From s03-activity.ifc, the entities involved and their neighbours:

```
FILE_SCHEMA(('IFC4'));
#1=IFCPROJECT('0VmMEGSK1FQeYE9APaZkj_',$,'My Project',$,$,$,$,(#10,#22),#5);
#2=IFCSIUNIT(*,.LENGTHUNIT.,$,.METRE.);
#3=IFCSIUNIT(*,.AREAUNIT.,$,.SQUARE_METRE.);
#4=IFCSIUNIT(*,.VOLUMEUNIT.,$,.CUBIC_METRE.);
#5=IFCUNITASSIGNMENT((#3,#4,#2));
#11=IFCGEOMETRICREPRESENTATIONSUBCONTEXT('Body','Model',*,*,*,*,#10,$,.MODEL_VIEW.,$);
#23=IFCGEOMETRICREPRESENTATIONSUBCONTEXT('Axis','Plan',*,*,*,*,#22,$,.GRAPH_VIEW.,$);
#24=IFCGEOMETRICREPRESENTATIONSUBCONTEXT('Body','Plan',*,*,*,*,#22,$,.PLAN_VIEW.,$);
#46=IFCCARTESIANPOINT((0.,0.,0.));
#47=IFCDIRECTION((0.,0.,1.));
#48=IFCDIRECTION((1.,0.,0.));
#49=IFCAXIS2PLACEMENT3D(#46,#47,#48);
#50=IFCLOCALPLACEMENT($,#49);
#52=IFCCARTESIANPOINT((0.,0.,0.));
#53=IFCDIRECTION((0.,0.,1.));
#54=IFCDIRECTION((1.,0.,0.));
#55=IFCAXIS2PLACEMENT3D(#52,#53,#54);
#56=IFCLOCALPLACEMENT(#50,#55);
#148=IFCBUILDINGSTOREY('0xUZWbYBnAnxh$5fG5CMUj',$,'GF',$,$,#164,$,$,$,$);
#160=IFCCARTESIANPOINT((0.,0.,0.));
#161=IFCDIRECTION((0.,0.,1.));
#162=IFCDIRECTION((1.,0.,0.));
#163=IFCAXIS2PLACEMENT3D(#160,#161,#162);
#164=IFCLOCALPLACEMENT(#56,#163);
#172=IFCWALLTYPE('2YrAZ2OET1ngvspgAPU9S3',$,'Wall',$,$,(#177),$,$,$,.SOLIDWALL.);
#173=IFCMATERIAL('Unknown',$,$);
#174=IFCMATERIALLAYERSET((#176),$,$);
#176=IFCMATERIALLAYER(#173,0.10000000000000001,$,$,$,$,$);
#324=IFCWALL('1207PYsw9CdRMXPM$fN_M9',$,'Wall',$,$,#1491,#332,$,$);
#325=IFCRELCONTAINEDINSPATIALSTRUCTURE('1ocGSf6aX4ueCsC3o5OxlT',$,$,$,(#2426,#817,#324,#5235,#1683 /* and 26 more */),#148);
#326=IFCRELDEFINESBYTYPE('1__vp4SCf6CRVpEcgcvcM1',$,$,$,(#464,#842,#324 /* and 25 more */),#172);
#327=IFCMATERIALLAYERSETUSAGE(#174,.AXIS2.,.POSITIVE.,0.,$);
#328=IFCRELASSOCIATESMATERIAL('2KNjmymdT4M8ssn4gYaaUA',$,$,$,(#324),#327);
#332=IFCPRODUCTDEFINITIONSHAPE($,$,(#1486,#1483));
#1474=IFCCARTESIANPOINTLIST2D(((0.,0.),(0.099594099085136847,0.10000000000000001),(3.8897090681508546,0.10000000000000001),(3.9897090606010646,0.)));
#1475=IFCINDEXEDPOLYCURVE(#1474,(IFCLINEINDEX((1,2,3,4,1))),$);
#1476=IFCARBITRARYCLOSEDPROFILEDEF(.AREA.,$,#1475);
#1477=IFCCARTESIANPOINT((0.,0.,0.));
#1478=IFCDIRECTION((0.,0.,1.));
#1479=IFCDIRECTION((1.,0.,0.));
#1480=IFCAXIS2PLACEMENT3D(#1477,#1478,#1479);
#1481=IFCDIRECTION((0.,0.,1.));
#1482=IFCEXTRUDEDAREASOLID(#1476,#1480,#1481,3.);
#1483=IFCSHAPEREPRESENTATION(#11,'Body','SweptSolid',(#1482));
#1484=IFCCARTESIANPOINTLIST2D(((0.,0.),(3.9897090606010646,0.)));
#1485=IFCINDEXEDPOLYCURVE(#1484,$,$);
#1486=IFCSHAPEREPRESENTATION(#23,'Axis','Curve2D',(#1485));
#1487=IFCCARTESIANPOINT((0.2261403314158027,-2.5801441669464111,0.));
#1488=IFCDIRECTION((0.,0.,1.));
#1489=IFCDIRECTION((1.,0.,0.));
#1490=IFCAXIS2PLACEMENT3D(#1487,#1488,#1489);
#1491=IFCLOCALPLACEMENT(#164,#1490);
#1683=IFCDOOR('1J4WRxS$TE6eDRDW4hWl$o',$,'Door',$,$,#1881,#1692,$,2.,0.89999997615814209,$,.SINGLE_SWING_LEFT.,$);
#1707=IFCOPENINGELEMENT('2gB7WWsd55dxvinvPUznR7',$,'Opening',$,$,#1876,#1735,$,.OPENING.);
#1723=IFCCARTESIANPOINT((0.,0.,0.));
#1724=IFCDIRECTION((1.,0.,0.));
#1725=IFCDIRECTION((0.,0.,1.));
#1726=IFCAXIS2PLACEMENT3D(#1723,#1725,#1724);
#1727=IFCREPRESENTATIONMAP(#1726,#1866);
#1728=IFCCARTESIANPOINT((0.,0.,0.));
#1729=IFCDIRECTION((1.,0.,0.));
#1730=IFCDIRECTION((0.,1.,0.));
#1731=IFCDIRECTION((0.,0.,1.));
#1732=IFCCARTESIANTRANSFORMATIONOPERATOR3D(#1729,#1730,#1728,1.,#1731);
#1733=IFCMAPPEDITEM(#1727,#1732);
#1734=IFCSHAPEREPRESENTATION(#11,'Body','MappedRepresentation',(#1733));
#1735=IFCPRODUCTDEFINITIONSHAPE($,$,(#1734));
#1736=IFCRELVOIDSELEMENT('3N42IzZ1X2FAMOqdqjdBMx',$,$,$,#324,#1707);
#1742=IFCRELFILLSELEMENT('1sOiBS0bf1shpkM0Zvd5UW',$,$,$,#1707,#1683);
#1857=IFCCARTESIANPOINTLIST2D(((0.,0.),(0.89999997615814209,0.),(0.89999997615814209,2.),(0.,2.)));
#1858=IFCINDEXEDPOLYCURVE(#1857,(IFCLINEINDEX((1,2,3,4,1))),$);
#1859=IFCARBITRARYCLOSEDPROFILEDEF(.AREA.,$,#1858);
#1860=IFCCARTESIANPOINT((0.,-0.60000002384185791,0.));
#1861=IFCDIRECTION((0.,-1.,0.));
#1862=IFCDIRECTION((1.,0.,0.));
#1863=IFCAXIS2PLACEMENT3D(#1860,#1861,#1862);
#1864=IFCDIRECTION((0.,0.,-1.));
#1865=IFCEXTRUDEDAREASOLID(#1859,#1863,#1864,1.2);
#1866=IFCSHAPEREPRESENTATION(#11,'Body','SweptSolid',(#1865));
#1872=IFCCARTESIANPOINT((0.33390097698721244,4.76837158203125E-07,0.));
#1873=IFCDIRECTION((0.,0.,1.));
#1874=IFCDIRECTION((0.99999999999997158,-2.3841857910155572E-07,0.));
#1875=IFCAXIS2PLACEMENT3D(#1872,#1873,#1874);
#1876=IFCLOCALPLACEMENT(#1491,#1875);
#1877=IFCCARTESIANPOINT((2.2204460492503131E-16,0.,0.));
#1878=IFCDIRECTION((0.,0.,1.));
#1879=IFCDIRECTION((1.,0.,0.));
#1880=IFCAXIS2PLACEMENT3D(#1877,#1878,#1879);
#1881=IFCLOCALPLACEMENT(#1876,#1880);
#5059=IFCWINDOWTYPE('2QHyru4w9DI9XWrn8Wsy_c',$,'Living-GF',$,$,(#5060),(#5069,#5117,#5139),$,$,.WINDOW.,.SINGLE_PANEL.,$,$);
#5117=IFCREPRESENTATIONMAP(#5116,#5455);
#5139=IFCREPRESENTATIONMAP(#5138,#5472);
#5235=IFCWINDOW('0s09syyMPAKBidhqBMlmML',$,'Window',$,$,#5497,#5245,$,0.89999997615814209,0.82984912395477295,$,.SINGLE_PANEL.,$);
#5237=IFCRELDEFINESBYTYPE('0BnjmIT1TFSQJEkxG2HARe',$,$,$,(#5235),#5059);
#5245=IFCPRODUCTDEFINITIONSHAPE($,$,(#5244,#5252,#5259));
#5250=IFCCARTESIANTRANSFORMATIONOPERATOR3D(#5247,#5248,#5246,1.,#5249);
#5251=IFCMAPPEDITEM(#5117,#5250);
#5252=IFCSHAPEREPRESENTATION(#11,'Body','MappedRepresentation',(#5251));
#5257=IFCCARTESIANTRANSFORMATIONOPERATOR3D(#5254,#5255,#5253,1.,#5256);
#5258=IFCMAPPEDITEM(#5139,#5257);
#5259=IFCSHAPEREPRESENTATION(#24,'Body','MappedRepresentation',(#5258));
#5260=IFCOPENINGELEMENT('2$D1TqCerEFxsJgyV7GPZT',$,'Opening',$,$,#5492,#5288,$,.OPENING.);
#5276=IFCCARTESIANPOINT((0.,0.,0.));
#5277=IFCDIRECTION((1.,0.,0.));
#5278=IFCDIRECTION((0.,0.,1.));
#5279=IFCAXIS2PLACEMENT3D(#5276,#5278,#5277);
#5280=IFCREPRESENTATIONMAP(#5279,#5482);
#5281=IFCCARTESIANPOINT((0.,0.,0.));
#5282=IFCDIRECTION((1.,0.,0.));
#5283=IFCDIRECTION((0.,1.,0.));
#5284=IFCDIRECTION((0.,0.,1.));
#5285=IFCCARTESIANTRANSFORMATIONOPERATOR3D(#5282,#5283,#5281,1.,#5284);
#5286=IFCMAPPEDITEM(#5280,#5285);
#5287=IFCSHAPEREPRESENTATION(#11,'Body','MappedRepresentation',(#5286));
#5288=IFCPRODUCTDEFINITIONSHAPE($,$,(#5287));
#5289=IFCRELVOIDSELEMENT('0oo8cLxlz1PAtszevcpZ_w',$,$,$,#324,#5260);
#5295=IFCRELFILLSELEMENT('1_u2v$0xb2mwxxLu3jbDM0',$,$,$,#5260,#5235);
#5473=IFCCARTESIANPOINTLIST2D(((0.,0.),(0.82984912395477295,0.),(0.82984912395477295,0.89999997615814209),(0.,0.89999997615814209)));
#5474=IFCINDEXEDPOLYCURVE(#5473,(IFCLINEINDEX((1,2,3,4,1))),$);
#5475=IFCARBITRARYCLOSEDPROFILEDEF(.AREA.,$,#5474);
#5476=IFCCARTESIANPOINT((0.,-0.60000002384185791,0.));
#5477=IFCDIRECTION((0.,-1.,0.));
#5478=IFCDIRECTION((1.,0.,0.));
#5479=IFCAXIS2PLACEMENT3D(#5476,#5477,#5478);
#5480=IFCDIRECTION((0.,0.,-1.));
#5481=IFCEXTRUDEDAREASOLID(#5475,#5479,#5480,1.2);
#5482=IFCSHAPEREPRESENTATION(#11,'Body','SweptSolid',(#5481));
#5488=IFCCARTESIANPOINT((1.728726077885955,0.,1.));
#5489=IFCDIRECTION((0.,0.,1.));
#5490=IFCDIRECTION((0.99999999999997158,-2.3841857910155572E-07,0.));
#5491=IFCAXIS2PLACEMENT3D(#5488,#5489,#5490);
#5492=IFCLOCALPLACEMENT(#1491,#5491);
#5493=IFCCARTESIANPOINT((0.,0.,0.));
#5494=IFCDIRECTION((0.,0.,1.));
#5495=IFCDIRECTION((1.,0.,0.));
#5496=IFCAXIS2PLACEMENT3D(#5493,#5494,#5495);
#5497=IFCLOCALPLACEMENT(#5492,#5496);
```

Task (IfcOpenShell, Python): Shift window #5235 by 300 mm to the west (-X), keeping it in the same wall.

```python
import ifcopenshell
import ifcopenshell.api.geometry
import ifcopenshell.util.placement
import ifcopenshell.util.unit

model = ifcopenshell.open("s03-activity.ifc")
unit_scale = ifcopenshell.util.unit.calculate_unit_scale(model)

window = model.by_id(5235)
opening = window.FillsVoids[0].RelatingOpeningElement
wall = opening.VoidsElements[0].RelatingBuildingElement

wall_matrix = ifcopenshell.util.placement.get_local_placement(wall.ObjectPlacement)
shift = wall_matrix[:3, 0] * -0.3 / unit_scale
before = ifcopenshell.util.placement.get_local_placement(window.ObjectPlacement)[:3, 3].copy()

# The window is placed relative to its opening, so it follows when the opening moves.
matrix = ifcopenshell.util.placement.get_local_placement(opening.ObjectPlacement)
matrix[:3, 3] += shift
ifcopenshell.api.geometry.edit_object_placement(
    model, product=opening, matrix=matrix, is_si=False, should_transform_children=True
)

after = ifcopenshell.util.placement.get_local_placement(window.ObjectPlacement)[:3, 3]
print("window moved by", (after - before).round(3) + 0.0)

model.write("s03-activity_rev.ifc")
```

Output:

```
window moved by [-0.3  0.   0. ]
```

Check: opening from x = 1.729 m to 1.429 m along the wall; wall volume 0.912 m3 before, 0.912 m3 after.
